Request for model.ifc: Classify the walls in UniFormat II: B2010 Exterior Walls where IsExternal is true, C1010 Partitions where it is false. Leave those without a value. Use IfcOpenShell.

First a look at what the model holds.

```python
import ifcopenshell
import ifcopenshell.util.element

model = ifcopenshell.open("model.ifc")
print(model.schema)
print("classifications:", [c.Name for c in model.by_type("IfcClassification")])
values = [ifcopenshell.util.element.get_pset(e, "Pset_WallCommon", "IsExternal") for e in model.by_type("IfcWall")]
for value in (True, False, None):
    print("IsExternal", value, values.count(value))
```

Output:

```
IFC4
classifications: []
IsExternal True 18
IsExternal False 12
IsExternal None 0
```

```python
import ifcopenshell
import ifcopenshell.api.classification
import ifcopenshell.util.element

model = ifcopenshell.open("model.ifc")

system = ifcopenshell.api.classification.add_classification(model, classification="UniFormat II")

walls = model.by_type("IfcWall")
external = {e: ifcopenshell.util.element.get_pset(e, "Pset_WallCommon", "IsExternal") for e in walls}
for flag, code, name in ((True, "B2010", "Exterior Walls"), (False, "C1010", "Partitions")):
    products = [e for e in walls if external[e] is flag]
    ifcopenshell.api.classification.add_reference(
        model, products=products, classification=system, identification=code, name=name
    )
    print(code, len(products))

model.write("model_updated.ifc")
```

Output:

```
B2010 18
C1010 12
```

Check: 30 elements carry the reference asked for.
